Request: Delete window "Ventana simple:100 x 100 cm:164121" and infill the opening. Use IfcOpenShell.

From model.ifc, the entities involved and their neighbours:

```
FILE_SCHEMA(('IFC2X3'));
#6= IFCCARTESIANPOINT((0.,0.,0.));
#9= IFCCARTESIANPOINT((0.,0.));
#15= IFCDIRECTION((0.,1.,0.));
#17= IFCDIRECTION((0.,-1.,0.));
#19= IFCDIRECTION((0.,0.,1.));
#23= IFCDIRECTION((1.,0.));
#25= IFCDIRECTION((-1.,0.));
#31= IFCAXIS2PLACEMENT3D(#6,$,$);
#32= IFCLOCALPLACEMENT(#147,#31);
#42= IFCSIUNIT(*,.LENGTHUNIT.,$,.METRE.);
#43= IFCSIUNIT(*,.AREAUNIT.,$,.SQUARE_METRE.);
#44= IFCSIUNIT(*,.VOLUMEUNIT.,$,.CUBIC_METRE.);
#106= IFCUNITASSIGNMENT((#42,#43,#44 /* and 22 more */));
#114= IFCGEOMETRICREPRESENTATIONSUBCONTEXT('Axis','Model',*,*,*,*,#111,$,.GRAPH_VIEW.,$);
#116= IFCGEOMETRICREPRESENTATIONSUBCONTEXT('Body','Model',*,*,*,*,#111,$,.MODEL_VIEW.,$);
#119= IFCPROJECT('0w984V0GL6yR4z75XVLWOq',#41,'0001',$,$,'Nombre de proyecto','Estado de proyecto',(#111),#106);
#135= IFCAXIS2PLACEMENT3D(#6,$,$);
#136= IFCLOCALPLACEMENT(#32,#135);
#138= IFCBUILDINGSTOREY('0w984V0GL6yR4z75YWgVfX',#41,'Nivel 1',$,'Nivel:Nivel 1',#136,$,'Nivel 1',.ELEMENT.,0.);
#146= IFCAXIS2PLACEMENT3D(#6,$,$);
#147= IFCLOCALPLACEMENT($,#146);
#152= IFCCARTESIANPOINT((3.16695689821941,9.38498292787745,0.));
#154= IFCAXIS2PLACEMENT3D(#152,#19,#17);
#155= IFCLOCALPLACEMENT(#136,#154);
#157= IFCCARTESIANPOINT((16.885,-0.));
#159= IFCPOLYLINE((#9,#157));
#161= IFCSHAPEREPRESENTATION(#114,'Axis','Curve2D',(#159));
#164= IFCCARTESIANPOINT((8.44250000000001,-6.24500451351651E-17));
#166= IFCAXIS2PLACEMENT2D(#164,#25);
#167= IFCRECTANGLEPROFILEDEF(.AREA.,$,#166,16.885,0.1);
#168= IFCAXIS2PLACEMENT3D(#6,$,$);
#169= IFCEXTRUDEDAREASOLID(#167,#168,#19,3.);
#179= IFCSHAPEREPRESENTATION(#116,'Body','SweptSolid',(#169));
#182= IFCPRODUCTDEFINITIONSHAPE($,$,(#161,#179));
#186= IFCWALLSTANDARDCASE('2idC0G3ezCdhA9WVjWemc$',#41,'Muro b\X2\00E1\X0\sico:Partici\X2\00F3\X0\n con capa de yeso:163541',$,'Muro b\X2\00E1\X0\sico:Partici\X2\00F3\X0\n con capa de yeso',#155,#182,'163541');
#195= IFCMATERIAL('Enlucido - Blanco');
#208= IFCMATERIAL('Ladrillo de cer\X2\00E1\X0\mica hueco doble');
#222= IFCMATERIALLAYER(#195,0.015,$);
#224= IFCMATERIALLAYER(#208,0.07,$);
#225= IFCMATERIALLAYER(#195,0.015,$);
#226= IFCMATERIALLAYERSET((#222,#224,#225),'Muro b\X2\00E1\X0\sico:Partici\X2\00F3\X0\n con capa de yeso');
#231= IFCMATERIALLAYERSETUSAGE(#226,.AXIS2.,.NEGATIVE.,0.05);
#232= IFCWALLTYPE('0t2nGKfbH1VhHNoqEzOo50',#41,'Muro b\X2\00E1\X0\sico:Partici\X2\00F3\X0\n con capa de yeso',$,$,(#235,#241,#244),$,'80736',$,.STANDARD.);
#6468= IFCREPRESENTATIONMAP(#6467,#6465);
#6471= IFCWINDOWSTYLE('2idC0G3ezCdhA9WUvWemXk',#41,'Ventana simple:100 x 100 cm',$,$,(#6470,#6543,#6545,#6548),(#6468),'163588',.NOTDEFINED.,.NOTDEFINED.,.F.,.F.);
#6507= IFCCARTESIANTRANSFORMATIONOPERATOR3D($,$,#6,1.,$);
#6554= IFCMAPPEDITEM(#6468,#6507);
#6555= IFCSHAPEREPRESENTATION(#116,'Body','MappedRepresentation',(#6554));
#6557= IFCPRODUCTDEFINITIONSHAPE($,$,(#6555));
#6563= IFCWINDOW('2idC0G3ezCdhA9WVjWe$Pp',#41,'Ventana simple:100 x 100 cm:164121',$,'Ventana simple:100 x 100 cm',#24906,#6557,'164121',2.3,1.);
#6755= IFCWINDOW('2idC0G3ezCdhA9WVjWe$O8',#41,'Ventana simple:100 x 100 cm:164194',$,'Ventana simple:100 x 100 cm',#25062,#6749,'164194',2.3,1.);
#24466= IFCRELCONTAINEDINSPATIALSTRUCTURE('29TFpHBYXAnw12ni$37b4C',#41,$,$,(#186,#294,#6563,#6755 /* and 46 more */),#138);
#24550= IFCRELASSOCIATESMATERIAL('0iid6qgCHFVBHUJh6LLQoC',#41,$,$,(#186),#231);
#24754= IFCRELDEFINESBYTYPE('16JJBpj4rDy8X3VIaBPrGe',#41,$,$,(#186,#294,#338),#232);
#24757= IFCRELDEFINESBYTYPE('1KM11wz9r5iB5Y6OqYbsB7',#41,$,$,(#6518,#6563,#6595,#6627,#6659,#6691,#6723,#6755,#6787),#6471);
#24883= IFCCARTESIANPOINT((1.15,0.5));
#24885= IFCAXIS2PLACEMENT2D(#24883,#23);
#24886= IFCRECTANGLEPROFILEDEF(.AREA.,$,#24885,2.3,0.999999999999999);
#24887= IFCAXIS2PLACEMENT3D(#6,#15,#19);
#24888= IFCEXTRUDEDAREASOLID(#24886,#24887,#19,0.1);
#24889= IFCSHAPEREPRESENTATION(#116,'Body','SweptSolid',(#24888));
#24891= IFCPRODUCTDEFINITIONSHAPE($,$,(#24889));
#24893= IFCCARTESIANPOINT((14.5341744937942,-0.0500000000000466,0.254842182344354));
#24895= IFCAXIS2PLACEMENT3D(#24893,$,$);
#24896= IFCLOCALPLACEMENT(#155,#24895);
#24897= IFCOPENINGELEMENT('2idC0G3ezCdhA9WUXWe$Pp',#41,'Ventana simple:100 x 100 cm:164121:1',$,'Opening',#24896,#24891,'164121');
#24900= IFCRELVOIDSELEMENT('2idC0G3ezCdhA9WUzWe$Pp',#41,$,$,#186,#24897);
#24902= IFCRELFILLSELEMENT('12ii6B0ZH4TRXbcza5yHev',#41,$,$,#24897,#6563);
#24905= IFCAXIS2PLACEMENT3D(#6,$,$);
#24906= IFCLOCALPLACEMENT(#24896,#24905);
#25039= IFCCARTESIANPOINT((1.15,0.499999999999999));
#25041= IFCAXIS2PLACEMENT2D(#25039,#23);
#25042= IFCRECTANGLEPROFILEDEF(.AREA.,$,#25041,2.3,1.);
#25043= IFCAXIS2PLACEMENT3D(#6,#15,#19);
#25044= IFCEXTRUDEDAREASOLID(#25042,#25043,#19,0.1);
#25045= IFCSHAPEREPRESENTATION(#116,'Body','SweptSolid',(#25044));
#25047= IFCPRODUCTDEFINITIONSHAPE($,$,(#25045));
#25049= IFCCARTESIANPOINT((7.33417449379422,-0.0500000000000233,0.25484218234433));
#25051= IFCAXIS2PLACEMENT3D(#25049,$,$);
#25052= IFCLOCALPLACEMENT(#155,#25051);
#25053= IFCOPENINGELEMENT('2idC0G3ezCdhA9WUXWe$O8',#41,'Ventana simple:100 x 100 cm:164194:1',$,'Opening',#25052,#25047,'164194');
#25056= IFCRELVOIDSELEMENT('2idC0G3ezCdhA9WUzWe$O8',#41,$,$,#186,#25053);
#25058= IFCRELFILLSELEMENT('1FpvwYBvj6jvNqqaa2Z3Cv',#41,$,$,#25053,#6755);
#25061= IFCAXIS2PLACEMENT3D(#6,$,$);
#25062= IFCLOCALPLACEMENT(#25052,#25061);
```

```python
import ifcopenshell
import ifcopenshell.api.feature
import ifcopenshell.api.root
import ifcopenshell.geom
import ifcopenshell.util.shape

model = ifcopenshell.open("model.ifc")
settings = ifcopenshell.geom.settings()


def volume(element):
    """Net volume in cubic metres, openings subtracted."""
    shape = ifcopenshell.geom.create_shape(settings, element)
    return ifcopenshell.util.shape.get_volume(shape.geometry)


window = model.by_guid("2idC0G3ezCdhA9WVjWe$Pp")
opening = window.FillsVoids[0].RelatingOpeningElement
wall = opening.VoidsElements[0].RelatingBuildingElement
before = volume(wall)

ifcopenshell.api.root.remove_product(model, product=window)
ifcopenshell.api.feature.remove_feature(model, feature=opening)

after = volume(wall)

print(f"wall volume {before:.3f} -> {after:.3f} m3")

model.write("model_rev.ifc")
```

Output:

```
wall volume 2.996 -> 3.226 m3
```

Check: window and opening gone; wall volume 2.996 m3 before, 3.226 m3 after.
